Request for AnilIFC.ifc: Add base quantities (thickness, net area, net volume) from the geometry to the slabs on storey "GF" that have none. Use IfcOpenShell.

First a look at what the model holds.

```python
import ifcopenshell
import ifcopenshell.util.element
import ifcopenshell.util.unit

model = ifcopenshell.open("AnilIFC.ifc")
print(model.schema)
for unit_type in ("LENGTHUNIT", "AREAUNIT", "VOLUMEUNIT"):
    print(unit_type, ifcopenshell.util.unit.calculate_unit_scale(model, unit_type))
storey = next(s for s in model.by_type("IfcBuildingStorey") if s.Name == "GF")
slabs = [e for e in ifcopenshell.util.element.get_decomposition(storey) if e.is_a("IfcSlab")]
for e in sorted(slabs, key=lambda e: e.id()):
    print(e.id(), e.is_a(), e.Name, list(ifcopenshell.util.element.get_psets(e, qtos_only=True)), sep=" | ")
```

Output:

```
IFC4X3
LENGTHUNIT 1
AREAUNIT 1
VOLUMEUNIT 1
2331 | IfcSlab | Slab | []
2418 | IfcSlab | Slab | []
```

```python
import ifcopenshell
import ifcopenshell.api.pset
import ifcopenshell.geom
import ifcopenshell.util.element
import ifcopenshell.util.shape
import ifcopenshell.util.unit

model = ifcopenshell.open("AnilIFC.ifc")
unit_scale = ifcopenshell.util.unit.calculate_unit_scale(model)
area_scale = ifcopenshell.util.unit.calculate_unit_scale(model, "AREAUNIT")
volume_scale = ifcopenshell.util.unit.calculate_unit_scale(model, "VOLUMEUNIT")
settings = ifcopenshell.geom.settings()

storey = next(s for s in model.by_type("IfcBuildingStorey") if s.Name == "GF")
slabs = [e for e in ifcopenshell.util.element.get_decomposition(storey) if e.is_a("IfcSlab")]

for e in sorted(slabs, key=lambda e: e.id()):
    if ifcopenshell.util.element.get_psets(e, qtos_only=True, should_inherit=False):
        continue
    # Geometry comes back in metres, in the element's own axes.
    shape = ifcopenshell.geom.create_shape(settings, e)
    values = {
        "Width": ifcopenshell.util.shape.get_z(shape.geometry) / unit_scale,
        "NetArea": ifcopenshell.util.shape.get_footprint_area(shape.geometry) / area_scale,
        "NetVolume": ifcopenshell.util.shape.get_volume(shape.geometry) / volume_scale,
    }
    qto = ifcopenshell.api.pset.add_qto(model, product=e, name="Qto_SlabBaseQuantities")
    ifcopenshell.api.pset.edit_qto(model, qto=qto, properties=values)
    print(e.id(), {k: round(v, 3) for k, v in values.items()})

model.write("AnilIFC-out.ifc")
```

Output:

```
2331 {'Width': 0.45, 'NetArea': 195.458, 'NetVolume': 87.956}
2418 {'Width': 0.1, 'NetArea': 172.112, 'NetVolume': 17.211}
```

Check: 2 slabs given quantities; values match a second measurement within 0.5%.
